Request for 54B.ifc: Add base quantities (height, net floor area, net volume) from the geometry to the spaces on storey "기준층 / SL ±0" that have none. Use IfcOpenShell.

First a look at what the model holds.

```python
import ifcopenshell
import ifcopenshell.util.element
import ifcopenshell.util.unit

model = ifcopenshell.open("54B.ifc")
print(model.schema)
for unit_type in ("LENGTHUNIT", "AREAUNIT", "VOLUMEUNIT"):
    print(unit_type, ifcopenshell.util.unit.calculate_unit_scale(model, unit_type))
storey = next(s for s in model.by_type("IfcBuildingStorey") if s.Name == "기준층 / SL ±0")
spaces = [e for e in ifcopenshell.util.element.get_decomposition(storey) if e.is_a("IfcSpace")]
for e in sorted(spaces, key=lambda e: e.id()):
    print(e.id(), e.is_a(), e.Name, list(ifcopenshell.util.element.get_psets(e, qtos_only=True)), sep=" | ")
```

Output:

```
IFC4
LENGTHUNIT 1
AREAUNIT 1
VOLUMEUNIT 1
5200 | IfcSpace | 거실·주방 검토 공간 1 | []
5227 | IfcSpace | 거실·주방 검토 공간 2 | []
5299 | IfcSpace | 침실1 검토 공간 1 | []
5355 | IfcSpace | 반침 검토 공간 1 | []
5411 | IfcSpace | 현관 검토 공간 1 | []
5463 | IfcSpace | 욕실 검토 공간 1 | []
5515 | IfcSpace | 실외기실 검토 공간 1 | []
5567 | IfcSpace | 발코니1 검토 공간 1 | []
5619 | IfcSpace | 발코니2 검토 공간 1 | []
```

```python
import ifcopenshell
import ifcopenshell.api.pset
import ifcopenshell.geom
import ifcopenshell.util.element
import ifcopenshell.util.shape
import ifcopenshell.util.unit

model = ifcopenshell.open("54B.ifc")
unit_scale = ifcopenshell.util.unit.calculate_unit_scale(model)
area_scale = ifcopenshell.util.unit.calculate_unit_scale(model, "AREAUNIT")
volume_scale = ifcopenshell.util.unit.calculate_unit_scale(model, "VOLUMEUNIT")
settings = ifcopenshell.geom.settings()

storey = next(s for s in model.by_type("IfcBuildingStorey") if s.Name == "기준층 / SL ±0")
spaces = [e for e in ifcopenshell.util.element.get_decomposition(storey) if e.is_a("IfcSpace")]

for e in sorted(spaces, key=lambda e: e.id()):
    if ifcopenshell.util.element.get_psets(e, qtos_only=True, should_inherit=False):
        continue
    # Geometry comes back in metres, in the element's own axes.
    shape = ifcopenshell.geom.create_shape(settings, e)
    values = {
        "Height": ifcopenshell.util.shape.get_z(shape.geometry) / unit_scale,
        "NetFloorArea": ifcopenshell.util.shape.get_footprint_area(shape.geometry) / area_scale,
        "NetVolume": ifcopenshell.util.shape.get_volume(shape.geometry) / volume_scale,
    }
    qto = ifcopenshell.api.pset.add_qto(model, product=e, name="Qto_SpaceBaseQuantities")
    ifcopenshell.api.pset.edit_qto(model, qto=qto, properties=values)
    print(e.id(), {k: round(v, 3) for k, v in values.items()})

model.write("54B_v2.ifc")
```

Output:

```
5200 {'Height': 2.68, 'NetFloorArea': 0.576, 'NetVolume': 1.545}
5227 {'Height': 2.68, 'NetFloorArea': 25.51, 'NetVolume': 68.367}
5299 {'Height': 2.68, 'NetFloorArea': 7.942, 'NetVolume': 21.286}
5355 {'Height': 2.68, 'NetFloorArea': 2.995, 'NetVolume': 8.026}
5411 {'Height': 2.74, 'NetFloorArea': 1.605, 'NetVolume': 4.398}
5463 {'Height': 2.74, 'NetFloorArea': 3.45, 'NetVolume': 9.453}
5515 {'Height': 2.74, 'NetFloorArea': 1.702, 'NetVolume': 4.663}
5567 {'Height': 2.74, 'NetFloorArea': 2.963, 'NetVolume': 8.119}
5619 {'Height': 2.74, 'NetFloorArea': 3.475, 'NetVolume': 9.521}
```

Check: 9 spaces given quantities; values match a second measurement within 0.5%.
